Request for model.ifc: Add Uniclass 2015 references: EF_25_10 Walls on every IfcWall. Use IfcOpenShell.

First a look at what the model holds.

```python
import ifcopenshell

model = ifcopenshell.open("model.ifc")
print(model.schema)
print("classifications:", [c.Name for c in model.by_type("IfcClassification")])
for ifc_class in ("IfcDoor", "IfcRoof", "IfcStair", "IfcWall", "IfcWindow"):
    print(ifc_class, len(model.by_type(ifc_class)))
```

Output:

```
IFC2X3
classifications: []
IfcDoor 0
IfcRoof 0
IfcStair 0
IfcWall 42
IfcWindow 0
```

```python
import ifcopenshell
import ifcopenshell.api.classification

model = ifcopenshell.open("model.ifc")

# IFC2X3 requires Source and Edition and has no link from the project to the system.
system = model.create_entity("IfcClassification", Source="NBS", Edition="2015", Name="Uniclass 2015")

codes = {
    "IfcWall": ("EF_25_10", "Walls"),
}
for ifc_class, (code, name) in codes.items():
    products = model.by_type(ifc_class)
    ifcopenshell.api.classification.add_reference(
        model, products=products, classification=system, identification=code, name=name
    )
    print(code, len(products))

model.write("model-out.ifc")
```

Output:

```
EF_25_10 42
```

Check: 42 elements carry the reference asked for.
